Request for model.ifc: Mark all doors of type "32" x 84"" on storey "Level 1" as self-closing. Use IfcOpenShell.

First a look at what the model holds.

```python
import ifcopenshell
import ifcopenshell.util.element

model = ifcopenshell.open("model.ifc")
print(model.schema)
storey = next(s for s in model.by_type("IfcBuildingStorey") if s.Name == "Level 1")
doors = [e for e in ifcopenshell.util.element.get_decomposition(storey) if e.is_a("IfcDoor")]
seen = {}
for e in doors:
    element_type = ifcopenshell.util.element.get_type(e)
    key = (element_type.Name if element_type != e and element_type else None, ifcopenshell.util.element.get_pset(e, "Pset_DoorCommon", "SelfClosing"))
    seen[key] = seen.get(key, 0) + 1
for (name, value), count in sorted(seen.items(), key=str):
    print(count, "x", name, "|", value)
```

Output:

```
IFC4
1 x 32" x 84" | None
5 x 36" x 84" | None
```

```python
import ifcopenshell
import ifcopenshell.api.pset
import ifcopenshell.util.element

model = ifcopenshell.open("model.ifc")

storey = next(s for s in model.by_type("IfcBuildingStorey") if s.Name == "Level 1")
doors = [e for e in ifcopenshell.util.element.get_decomposition(storey) if e.is_a("IfcDoor")]

count = 0
for e in doors:
    element_type = ifcopenshell.util.element.get_type(e)
    if element_type in (None, e) or element_type.Name != '32" x 84"':
        continue
    # add_pset returns the element's existing set when there is one.
    pset = ifcopenshell.api.pset.add_pset(model, product=e, name="Pset_DoorCommon")
    ifcopenshell.api.pset.edit_pset(model, pset=pset, properties={"SelfClosing": True})
    count += 1

print(count, "doors updated")

model.write("model_v2.ifc")
```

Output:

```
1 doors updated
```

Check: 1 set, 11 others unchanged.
